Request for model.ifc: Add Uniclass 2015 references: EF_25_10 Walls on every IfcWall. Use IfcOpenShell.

First a look at what the model holds.

```python
import ifcopenshell

model = ifcopenshell.open("model.ifc")
print(model.schema)
print("classifications:", [c.Name for c in model.by_type("IfcClassification")])
for ifc_class in ("IfcDoor", "IfcRoof", "IfcStair", "IfcWall", "IfcWindow"):
    print(ifc_class, len(model.by_type(ifc_class)))
```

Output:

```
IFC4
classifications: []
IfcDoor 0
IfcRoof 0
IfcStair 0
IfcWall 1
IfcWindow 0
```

```python
import ifcopenshell
import ifcopenshell.api.classification

model = ifcopenshell.open("model.ifc")

system = ifcopenshell.api.classification.add_classification(model, classification="Uniclass 2015")

codes = {
    "IfcWall": ("EF_25_10", "Walls"),
}
for ifc_class, (code, name) in codes.items():
    products = model.by_type(ifc_class)
    ifcopenshell.api.classification.add_reference(
        model, products=products, classification=system, identification=code, name=name
    )
    print(code, len(products))

model.write("model_rev.ifc")
```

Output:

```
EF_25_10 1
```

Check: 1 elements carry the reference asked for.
